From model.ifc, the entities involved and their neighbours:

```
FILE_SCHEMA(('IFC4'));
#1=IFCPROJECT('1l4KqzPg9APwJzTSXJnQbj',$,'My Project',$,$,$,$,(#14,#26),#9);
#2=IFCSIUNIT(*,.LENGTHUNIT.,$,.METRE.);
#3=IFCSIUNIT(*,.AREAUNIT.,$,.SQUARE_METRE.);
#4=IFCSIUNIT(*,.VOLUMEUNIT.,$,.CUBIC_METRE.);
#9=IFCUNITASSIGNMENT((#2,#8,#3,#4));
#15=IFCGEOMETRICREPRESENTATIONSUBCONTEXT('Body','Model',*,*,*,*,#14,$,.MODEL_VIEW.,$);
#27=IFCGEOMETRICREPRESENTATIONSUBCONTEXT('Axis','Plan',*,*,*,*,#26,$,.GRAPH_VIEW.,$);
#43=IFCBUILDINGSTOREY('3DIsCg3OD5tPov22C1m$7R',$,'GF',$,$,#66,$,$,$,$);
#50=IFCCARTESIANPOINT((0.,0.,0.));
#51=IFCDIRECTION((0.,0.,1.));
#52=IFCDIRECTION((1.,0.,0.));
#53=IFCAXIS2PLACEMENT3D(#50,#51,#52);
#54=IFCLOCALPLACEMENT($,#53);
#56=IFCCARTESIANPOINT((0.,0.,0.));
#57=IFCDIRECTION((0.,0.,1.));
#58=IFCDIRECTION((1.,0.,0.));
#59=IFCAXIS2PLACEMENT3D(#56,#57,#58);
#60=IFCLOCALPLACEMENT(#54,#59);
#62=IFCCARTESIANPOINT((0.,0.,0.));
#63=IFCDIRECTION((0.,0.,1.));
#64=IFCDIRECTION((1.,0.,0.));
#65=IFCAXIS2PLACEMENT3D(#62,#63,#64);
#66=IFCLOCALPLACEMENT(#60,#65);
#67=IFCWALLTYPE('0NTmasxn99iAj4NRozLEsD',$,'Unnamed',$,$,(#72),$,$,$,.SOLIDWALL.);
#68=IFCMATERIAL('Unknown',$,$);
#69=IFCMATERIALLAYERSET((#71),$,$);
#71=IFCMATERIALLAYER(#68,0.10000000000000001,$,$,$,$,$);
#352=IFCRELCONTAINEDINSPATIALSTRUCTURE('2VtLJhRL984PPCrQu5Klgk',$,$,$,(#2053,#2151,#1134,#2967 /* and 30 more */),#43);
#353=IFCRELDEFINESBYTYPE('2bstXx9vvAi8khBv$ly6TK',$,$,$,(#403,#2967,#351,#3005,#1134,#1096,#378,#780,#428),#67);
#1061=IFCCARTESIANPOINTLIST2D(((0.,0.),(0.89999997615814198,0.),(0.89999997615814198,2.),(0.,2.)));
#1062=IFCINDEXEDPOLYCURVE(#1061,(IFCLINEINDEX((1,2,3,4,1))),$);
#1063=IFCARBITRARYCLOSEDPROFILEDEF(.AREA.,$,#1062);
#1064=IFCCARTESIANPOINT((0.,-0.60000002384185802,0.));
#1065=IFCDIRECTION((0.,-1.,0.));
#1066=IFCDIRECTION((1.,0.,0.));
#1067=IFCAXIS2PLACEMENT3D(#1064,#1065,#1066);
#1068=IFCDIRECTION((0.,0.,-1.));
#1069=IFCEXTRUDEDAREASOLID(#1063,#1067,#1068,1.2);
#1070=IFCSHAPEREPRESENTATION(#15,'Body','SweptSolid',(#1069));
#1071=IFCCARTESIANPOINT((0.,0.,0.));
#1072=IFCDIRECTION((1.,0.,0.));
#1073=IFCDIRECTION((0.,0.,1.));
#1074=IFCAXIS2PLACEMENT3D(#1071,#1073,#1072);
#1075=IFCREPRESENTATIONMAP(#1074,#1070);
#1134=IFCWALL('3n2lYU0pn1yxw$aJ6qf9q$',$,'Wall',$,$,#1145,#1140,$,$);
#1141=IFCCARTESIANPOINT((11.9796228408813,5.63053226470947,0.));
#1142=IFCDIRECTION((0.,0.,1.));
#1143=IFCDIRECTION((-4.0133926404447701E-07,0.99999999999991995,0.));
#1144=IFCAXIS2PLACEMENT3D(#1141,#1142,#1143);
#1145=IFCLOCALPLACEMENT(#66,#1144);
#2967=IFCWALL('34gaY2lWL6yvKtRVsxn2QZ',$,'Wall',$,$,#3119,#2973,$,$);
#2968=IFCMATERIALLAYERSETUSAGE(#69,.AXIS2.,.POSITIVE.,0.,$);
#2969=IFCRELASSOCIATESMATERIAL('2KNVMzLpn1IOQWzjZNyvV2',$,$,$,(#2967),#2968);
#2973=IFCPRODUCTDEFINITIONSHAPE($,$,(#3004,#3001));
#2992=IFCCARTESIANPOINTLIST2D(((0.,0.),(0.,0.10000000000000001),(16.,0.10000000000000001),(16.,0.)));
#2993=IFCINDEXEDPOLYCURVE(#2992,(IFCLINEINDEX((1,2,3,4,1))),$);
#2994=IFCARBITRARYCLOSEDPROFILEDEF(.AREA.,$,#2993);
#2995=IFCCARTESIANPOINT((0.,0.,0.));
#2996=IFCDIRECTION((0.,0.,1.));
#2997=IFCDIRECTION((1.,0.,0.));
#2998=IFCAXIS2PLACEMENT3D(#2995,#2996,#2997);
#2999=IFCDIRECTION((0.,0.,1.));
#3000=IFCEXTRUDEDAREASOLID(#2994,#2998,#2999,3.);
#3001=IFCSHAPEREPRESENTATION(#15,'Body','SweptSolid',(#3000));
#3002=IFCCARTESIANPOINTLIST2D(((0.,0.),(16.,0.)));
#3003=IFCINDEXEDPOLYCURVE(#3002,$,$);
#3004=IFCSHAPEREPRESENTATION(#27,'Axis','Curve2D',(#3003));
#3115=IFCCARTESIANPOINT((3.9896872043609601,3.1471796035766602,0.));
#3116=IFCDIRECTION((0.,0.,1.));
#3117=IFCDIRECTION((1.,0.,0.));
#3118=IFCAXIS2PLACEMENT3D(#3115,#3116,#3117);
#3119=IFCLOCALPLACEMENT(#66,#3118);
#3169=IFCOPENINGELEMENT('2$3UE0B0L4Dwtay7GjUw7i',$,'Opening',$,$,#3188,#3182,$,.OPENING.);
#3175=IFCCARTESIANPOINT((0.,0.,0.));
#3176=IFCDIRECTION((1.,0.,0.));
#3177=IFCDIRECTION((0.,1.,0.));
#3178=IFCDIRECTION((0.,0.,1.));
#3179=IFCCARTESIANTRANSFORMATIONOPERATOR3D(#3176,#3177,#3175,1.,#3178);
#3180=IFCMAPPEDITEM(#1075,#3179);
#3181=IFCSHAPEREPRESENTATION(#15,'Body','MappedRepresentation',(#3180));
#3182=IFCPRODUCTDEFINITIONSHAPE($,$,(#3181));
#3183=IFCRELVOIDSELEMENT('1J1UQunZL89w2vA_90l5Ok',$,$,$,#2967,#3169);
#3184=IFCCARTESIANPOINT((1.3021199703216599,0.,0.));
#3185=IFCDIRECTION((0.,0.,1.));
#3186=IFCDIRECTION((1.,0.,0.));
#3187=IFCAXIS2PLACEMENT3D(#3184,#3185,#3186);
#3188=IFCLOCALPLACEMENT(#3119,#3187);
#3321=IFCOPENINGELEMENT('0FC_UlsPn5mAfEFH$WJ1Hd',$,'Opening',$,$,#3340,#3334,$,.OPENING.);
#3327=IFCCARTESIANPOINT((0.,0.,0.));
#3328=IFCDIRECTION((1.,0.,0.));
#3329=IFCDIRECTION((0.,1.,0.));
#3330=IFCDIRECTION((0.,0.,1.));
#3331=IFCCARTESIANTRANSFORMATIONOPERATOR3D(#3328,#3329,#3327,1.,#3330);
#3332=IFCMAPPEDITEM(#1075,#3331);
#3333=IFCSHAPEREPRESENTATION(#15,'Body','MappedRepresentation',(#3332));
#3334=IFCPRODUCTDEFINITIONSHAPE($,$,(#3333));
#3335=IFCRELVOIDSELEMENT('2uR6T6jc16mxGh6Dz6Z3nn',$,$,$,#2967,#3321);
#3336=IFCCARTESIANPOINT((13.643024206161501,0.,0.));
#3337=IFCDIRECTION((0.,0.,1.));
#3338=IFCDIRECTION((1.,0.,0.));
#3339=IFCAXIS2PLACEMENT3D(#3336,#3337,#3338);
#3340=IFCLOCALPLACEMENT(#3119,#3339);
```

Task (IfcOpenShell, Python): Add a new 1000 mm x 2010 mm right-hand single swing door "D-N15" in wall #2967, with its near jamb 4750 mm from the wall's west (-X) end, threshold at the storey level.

```python
import numpy as np
import ifcopenshell
import ifcopenshell.api.feature
import ifcopenshell.api.geometry
import ifcopenshell.api.root
import ifcopenshell.api.spatial
import ifcopenshell.geom
import ifcopenshell.util.element
import ifcopenshell.util.placement
import ifcopenshell.util.representation
import ifcopenshell.util.shape
import ifcopenshell.util.unit

model = ifcopenshell.open("model.ifc")
unit_scale = ifcopenshell.util.unit.calculate_unit_scale(model)
settings = ifcopenshell.geom.settings()


def volume(element):
    """Net volume in cubic metres, openings subtracted."""
    shape = ifcopenshell.geom.create_shape(settings, element)
    return ifcopenshell.util.shape.get_volume(shape.geometry)


wall = model.by_id(2967)
storey = ifcopenshell.util.element.get_container(wall, ifc_class="IfcBuildingStorey")
context = ifcopenshell.util.representation.get_context(model, "Model", "Body", "MODEL_VIEW")
before = volume(wall)

width, height, from_end, sill = 1, 2.01, 4.75, 0.0  # metres

# The wall runs along its own X axis, and the end named is its -X end.
wall_shape = ifcopenshell.geom.create_shape(settings, wall)
x, y, z = ifcopenshell.util.shape.get_vertices(wall_shape.geometry).T
start = x.min() + from_end
face, thickness = float(y.min()), float(y.max() - y.min())
wall_matrix = ifcopenshell.util.placement.get_local_placement(wall.ObjectPlacement)
level = ifcopenshell.util.placement.get_local_placement(storey.ObjectPlacement)[2, 3]


def in_wall(x, y):
    """Placement at x, y metres in the wall's axes, at sill height."""
    matrix = wall_matrix.copy()
    matrix[:, 3] = wall_matrix @ np.array([x / unit_scale, y / unit_scale, 0.0, 1.0])
    matrix[2, 3] = level + sill / unit_scale
    return matrix


# Opening: a box that overshoots both wall faces by 50 mm.
opening = ifcopenshell.api.root.create_entity(model, ifc_class="IfcOpeningElement", predefined_type="OPENING")
box = ifcopenshell.api.geometry.add_wall_representation(
    model, context=context, length=width, height=height, thickness=thickness + 0.1
)
ifcopenshell.api.geometry.assign_representation(model, product=opening, representation=box)
ifcopenshell.api.geometry.edit_object_placement(model, product=opening, matrix=in_wall(start, face - 0.05), is_si=False)
ifcopenshell.api.feature.add_feature(model, feature=opening, element=wall)

door = ifcopenshell.api.root.create_entity(model, ifc_class="IfcDoor", name="D-N15", predefined_type="DOOR")
door.OverallWidth, door.OverallHeight = width / unit_scale, height / unit_scale
door.OperationType = "SINGLE_SWING_RIGHT"
body = ifcopenshell.api.geometry.add_door_representation(
    model,
    context=context,
    overall_width=door.OverallWidth,
    overall_height=door.OverallHeight,
    operation_type="SINGLE_SWING_RIGHT",
    lining_properties={"LiningDepth": thickness / unit_scale, "ThresholdDepth": thickness / unit_scale},
)
ifcopenshell.api.geometry.assign_representation(model, product=door, representation=body)
ifcopenshell.api.spatial.assign_container(model, products=[door], relating_structure=storey)
ifcopenshell.api.feature.add_filling(model, opening=opening, element=door)

# The lining spans the wall, so the door starts at the wall face.
ifcopenshell.api.geometry.edit_object_placement(model, product=door, matrix=in_wall(start, face), is_si=False)

after = volume(wall)

print(f"wall volume {before:.3f} -> {after:.3f} m3")

model.write("model_v2.ifc")
```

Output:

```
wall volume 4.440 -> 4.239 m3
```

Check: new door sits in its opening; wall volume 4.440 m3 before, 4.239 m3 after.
